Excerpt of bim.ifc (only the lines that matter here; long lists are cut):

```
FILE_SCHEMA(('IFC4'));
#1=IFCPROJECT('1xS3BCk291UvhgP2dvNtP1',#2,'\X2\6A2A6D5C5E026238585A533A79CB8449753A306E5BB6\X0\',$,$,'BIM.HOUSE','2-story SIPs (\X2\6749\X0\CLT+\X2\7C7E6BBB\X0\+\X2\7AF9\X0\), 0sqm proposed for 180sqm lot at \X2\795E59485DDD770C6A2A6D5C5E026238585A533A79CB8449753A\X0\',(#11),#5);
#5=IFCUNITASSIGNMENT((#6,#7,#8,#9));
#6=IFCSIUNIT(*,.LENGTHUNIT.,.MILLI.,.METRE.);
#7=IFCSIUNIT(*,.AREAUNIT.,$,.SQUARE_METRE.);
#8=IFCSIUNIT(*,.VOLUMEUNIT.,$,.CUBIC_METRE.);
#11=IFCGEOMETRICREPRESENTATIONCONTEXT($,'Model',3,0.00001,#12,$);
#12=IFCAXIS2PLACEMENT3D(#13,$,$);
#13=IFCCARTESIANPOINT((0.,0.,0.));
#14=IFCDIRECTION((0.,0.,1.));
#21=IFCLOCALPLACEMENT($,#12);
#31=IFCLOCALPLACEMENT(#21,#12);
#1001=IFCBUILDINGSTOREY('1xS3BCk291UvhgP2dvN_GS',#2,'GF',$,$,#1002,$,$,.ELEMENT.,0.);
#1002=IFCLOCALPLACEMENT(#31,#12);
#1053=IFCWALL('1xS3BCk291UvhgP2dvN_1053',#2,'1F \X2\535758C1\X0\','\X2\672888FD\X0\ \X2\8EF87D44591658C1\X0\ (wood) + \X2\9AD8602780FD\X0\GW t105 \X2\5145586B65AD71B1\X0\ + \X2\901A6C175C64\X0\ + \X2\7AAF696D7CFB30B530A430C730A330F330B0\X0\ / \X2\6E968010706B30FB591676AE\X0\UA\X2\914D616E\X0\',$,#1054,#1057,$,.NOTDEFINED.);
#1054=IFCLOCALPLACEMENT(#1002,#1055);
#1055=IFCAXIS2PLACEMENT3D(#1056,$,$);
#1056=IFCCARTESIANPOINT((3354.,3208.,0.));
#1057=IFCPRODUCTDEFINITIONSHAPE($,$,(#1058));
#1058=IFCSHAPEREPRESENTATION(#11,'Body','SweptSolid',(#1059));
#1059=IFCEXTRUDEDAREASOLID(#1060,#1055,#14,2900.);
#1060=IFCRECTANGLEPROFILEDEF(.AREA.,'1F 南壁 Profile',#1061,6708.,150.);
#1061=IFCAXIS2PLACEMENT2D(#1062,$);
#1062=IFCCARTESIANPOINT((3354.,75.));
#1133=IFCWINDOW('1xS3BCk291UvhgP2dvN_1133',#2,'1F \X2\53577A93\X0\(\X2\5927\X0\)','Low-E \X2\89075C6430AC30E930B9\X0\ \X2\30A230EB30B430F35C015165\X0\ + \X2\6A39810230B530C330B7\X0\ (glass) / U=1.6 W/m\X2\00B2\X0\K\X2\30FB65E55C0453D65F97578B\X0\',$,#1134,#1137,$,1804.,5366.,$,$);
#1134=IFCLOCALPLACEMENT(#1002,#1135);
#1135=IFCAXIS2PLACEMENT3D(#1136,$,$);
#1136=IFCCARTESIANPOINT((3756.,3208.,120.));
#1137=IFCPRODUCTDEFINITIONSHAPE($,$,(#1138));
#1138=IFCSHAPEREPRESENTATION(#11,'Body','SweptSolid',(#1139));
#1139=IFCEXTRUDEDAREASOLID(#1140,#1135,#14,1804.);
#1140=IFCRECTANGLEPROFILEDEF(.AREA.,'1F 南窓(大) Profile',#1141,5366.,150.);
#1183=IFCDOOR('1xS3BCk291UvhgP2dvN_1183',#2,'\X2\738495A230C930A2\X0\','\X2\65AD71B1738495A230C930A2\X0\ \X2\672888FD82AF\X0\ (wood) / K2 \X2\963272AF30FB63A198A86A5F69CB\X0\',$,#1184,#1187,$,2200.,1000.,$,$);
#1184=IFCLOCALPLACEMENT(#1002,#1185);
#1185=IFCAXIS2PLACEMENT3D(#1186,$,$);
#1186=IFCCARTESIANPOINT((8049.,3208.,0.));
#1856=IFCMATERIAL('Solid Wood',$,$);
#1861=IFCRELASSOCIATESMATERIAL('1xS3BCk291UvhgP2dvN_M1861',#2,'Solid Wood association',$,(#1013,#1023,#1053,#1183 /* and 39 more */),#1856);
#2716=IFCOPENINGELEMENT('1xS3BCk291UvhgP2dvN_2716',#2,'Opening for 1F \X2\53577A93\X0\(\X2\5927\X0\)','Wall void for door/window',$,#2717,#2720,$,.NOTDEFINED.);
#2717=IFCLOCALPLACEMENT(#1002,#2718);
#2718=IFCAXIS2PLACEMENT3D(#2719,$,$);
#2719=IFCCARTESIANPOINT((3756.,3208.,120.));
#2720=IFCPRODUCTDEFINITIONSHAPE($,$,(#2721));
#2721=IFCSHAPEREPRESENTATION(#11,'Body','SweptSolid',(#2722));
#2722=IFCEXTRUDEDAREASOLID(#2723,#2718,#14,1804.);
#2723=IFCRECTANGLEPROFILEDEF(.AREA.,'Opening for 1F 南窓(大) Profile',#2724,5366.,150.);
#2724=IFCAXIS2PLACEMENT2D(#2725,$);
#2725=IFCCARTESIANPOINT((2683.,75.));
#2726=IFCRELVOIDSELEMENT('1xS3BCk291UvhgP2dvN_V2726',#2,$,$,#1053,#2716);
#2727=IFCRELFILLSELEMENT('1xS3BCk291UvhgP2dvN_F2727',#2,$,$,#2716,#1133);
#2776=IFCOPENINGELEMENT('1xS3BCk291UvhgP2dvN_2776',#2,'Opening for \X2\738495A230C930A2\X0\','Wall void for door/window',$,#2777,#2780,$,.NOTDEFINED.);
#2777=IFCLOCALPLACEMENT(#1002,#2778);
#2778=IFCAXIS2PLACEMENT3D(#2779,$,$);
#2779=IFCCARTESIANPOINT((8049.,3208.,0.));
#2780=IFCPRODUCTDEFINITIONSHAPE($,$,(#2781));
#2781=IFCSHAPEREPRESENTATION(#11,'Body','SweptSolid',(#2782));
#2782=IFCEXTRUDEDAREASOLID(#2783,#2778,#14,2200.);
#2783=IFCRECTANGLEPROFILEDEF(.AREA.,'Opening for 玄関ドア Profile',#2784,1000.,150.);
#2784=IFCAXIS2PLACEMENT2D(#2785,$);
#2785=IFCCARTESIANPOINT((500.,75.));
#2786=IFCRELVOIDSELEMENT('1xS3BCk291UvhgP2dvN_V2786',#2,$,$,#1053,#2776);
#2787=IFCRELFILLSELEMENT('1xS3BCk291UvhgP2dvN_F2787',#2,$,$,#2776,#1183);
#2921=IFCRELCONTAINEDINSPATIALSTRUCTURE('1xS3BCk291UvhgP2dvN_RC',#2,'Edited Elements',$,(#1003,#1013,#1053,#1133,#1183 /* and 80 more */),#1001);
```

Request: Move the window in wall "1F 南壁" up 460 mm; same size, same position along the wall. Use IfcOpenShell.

```python
import numpy as np
import ifcopenshell
import ifcopenshell.api.geometry
import ifcopenshell.util.placement
import ifcopenshell.util.unit

model = ifcopenshell.open("bim.ifc")
unit_scale = ifcopenshell.util.unit.calculate_unit_scale(model)

window = model.by_id(1133)
opening = window.FillsVoids[0].RelatingOpeningElement
dz = 0.46 / unit_scale

shift = np.array([0.0, 0.0, dz])
# The window is not placed relative to its opening, so move both.
for product in (opening, window):
    matrix = ifcopenshell.util.placement.get_local_placement(product.ObjectPlacement)
    matrix[:3, 3] += shift
    ifcopenshell.api.geometry.edit_object_placement(model, product=product, matrix=matrix, is_si=False)

print(f"moved by {dz * unit_scale:+.3f} m")

model.write("bim_rev.ifc")
```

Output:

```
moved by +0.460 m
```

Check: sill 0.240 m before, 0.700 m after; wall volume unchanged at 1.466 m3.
